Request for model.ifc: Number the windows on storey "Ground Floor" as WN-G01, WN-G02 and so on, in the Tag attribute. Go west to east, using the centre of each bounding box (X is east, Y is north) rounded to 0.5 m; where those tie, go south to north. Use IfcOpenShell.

First a look at what the model holds.

```python
import ifcopenshell
import ifcopenshell.util.element
import ifcopenshell.util.placement

model = ifcopenshell.open("model.ifc")
print(model.schema)
storey = next(s for s in model.by_type("IfcBuildingStorey") if s.Name == "Ground Floor")
windows = [e for e in ifcopenshell.util.element.get_decomposition(storey) if e.is_a("IfcWindow")]
for e in sorted(windows, key=lambda e: e.id()):
    origin = ifcopenshell.util.placement.get_local_placement(e.ObjectPlacement)[:3, 3]
    print(e.id(), e.Tag, e.Name, origin.round(2) + 0.0, sep=" | ")
```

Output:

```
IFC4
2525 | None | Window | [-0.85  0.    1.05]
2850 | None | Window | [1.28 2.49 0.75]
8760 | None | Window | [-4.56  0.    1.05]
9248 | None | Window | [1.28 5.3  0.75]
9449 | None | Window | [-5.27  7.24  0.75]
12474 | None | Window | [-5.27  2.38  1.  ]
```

```python
import ifcopenshell
import ifcopenshell.geom
import ifcopenshell.util.element
import ifcopenshell.util.shape

model = ifcopenshell.open("model.ifc")
settings = ifcopenshell.geom.settings()
settings.set("use-world-coords", True)


def centre(element):
    shape = ifcopenshell.geom.create_shape(settings, element)
    return ifcopenshell.util.shape.get_bbox_centroid(shape.geometry)


storey = next(s for s in model.by_type("IfcBuildingStorey") if s.Name == "Ground Floor")
windows = [e for e in ifcopenshell.util.element.get_decomposition(storey) if e.is_a("IfcWindow")]

# Insertion points can sit at a corner or the storey origin, so sort by the geometry (in metres).
centres = {e: centre(e) for e in windows}
windows.sort(key=lambda e: (round(centres[e][0] / 0.5), centres[e][1]))

for i, e in enumerate(windows, start=1):
    number = f"WN-G{i:02d}"
    e.Tag = number
    print(e.id(), number)

model.write("model_updated.ifc")
```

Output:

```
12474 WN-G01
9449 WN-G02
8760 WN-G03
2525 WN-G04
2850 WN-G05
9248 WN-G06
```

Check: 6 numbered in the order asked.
